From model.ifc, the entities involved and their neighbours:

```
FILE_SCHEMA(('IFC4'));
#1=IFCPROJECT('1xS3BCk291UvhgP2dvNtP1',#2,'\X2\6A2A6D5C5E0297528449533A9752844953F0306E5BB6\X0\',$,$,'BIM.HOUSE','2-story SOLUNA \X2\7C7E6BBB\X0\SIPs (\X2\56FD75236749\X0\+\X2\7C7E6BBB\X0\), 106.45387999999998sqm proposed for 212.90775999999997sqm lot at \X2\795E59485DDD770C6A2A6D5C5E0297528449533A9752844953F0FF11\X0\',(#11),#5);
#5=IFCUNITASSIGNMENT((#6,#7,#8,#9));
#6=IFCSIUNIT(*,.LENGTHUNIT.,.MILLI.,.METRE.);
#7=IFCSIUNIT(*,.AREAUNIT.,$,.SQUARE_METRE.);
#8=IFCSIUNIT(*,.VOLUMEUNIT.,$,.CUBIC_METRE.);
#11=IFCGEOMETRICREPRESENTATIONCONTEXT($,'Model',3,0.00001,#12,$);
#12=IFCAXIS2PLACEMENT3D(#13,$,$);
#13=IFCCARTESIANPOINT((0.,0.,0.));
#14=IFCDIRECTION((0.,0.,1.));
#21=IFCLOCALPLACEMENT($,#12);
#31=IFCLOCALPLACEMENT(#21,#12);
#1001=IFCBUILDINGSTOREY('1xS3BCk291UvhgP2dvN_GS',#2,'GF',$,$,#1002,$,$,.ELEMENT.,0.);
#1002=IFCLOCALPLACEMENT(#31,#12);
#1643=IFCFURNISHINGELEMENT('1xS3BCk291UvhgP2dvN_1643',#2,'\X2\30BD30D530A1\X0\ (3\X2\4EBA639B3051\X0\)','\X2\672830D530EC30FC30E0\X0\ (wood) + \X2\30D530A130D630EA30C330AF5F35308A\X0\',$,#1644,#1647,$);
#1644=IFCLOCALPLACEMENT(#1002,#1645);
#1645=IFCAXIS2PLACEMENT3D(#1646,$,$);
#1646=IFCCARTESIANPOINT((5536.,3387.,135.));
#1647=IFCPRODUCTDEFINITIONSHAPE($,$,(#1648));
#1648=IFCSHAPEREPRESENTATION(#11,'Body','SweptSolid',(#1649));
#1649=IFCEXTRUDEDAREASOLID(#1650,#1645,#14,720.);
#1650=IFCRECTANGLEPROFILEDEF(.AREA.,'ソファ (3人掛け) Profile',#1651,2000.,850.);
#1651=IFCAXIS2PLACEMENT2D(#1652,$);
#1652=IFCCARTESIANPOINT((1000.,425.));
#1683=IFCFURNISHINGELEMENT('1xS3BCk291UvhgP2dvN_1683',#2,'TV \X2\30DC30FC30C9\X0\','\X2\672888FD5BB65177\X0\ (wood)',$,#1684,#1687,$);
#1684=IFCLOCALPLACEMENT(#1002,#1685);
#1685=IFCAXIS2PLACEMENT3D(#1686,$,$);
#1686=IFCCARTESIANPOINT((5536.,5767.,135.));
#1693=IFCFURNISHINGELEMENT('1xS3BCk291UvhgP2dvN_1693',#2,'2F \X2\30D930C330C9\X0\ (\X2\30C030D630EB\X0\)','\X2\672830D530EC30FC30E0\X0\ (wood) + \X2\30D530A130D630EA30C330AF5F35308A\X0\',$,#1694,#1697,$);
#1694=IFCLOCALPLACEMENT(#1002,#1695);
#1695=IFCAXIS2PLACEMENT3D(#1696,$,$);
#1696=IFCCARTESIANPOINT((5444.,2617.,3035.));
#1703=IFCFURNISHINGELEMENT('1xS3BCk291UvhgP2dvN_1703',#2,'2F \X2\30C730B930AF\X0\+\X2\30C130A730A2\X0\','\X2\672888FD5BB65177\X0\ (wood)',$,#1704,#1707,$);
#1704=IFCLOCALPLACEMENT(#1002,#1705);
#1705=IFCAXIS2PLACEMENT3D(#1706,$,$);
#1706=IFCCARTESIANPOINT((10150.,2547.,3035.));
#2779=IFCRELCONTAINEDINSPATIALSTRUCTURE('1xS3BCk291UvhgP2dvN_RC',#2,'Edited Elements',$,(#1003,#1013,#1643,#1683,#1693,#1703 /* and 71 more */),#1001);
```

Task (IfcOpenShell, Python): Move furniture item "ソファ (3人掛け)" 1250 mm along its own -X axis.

```python
import ifcopenshell
import ifcopenshell.api.geometry
import ifcopenshell.util.placement

model = ifcopenshell.open("model.ifc")

item = model.by_guid("1xS3BCk291UvhgP2dvN_1643")
matrix = ifcopenshell.util.placement.get_local_placement(item.ObjectPlacement)
matrix[:3, 3] -= matrix[:3, 0] * 1250.0
ifcopenshell.api.geometry.edit_object_placement(model, product=item, matrix=matrix, is_si=False)

print(ifcopenshell.util.placement.get_local_placement(item.ObjectPlacement).round(3) + 0.0)

model.write("model-out.ifc")
```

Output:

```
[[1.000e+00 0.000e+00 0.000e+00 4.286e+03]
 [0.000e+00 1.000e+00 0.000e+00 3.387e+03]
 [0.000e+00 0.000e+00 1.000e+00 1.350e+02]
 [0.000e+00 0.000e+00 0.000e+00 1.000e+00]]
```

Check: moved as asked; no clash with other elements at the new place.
